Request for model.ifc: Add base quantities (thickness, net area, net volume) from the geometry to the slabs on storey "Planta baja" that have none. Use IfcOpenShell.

First a look at what the model holds.

```python
import ifcopenshell
import ifcopenshell.util.element
import ifcopenshell.util.unit

model = ifcopenshell.open("model.ifc")
print(model.schema)
for unit_type in ("LENGTHUNIT", "AREAUNIT", "VOLUMEUNIT"):
    print(unit_type, ifcopenshell.util.unit.calculate_unit_scale(model, unit_type))
storey = next(s for s in model.by_type("IfcBuildingStorey") if s.Name == "Planta baja")
slabs = [e for e in ifcopenshell.util.element.get_decomposition(storey) if e.is_a("IfcSlab")]
for e in sorted(slabs, key=lambda e: e.id()):
    print(e.id(), e.is_a(), e.Name, list(ifcopenshell.util.element.get_psets(e, qtos_only=True)), sep=" | ")
```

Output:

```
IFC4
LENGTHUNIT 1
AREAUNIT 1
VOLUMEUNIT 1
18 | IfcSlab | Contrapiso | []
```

```python
import ifcopenshell
import ifcopenshell.api.pset
import ifcopenshell.geom
import ifcopenshell.util.element
import ifcopenshell.util.shape
import ifcopenshell.util.unit

model = ifcopenshell.open("model.ifc")
unit_scale = ifcopenshell.util.unit.calculate_unit_scale(model)
area_scale = ifcopenshell.util.unit.calculate_unit_scale(model, "AREAUNIT")
volume_scale = ifcopenshell.util.unit.calculate_unit_scale(model, "VOLUMEUNIT")
settings = ifcopenshell.geom.settings()

storey = next(s for s in model.by_type("IfcBuildingStorey") if s.Name == "Planta baja")
slabs = [e for e in ifcopenshell.util.element.get_decomposition(storey) if e.is_a("IfcSlab")]

for e in sorted(slabs, key=lambda e: e.id()):
    if ifcopenshell.util.element.get_psets(e, qtos_only=True, should_inherit=False):
        continue
    # Geometry comes back in metres, in the element's own axes.
    shape = ifcopenshell.geom.create_shape(settings, e)
    values = {
        "Width": ifcopenshell.util.shape.get_z(shape.geometry) / unit_scale,
        "NetArea": ifcopenshell.util.shape.get_footprint_area(shape.geometry) / area_scale,
        "NetVolume": ifcopenshell.util.shape.get_volume(shape.geometry) / volume_scale,
    }
    qto = ifcopenshell.api.pset.add_qto(model, product=e, name="Qto_SlabBaseQuantities")
    ifcopenshell.api.pset.edit_qto(model, qto=qto, properties=values)
    print(e.id(), {k: round(v, 3) for k, v in values.items()})

model.write("model-out.ifc")
```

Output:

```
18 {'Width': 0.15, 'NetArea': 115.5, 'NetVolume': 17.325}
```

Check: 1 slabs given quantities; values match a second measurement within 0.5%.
